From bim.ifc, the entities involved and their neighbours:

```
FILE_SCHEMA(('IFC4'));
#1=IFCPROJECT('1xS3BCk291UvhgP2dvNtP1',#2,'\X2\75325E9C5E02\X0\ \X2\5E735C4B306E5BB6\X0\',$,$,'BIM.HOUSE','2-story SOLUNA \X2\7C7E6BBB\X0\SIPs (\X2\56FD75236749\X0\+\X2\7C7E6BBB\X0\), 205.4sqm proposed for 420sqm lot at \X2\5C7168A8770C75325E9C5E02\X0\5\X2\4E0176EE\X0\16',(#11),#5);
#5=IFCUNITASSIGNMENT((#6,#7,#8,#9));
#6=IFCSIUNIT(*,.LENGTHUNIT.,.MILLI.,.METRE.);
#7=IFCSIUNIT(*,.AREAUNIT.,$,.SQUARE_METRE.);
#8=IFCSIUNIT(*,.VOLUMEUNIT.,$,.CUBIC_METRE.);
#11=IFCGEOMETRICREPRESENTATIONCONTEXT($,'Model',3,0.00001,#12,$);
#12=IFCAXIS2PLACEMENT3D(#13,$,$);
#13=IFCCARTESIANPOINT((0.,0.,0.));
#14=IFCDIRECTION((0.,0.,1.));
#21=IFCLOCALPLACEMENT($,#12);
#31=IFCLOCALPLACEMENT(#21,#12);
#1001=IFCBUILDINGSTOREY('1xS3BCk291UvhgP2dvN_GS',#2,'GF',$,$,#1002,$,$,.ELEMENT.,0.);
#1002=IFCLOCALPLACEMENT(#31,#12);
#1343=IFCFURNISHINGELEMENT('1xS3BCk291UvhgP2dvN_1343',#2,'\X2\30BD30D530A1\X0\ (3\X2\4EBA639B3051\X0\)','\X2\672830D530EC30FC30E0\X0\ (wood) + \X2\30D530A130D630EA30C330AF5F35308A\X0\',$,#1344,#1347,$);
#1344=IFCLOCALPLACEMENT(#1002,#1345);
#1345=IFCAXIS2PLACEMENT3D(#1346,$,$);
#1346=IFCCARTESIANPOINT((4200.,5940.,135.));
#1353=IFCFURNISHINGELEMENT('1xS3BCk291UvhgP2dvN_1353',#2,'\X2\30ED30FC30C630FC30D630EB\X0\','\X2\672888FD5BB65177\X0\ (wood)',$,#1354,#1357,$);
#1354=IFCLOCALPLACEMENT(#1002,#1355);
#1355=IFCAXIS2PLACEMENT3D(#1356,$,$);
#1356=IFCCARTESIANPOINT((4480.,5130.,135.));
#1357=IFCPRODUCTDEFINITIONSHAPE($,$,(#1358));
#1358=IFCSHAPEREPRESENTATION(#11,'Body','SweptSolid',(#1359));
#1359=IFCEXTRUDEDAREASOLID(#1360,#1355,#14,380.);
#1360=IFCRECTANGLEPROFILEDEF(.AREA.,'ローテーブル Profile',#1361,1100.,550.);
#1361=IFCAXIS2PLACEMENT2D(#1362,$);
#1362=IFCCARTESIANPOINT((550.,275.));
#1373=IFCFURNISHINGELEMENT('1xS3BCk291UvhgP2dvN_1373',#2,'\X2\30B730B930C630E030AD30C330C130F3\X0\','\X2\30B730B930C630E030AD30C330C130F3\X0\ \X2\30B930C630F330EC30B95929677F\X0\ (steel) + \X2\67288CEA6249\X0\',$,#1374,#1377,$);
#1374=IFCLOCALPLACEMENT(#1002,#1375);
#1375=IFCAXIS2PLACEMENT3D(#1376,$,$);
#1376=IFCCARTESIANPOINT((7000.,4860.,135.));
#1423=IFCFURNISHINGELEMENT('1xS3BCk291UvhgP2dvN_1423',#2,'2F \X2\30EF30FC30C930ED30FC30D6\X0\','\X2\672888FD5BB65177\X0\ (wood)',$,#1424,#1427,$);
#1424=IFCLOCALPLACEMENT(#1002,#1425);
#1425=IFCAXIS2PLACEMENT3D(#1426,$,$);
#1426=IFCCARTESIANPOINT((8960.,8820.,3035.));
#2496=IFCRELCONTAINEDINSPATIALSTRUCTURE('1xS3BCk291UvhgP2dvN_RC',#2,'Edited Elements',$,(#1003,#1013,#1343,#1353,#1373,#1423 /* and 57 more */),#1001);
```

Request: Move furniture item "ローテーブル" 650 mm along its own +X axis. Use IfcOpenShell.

```python
import ifcopenshell
import ifcopenshell.api.geometry
import ifcopenshell.util.placement

model = ifcopenshell.open("bim.ifc")

item = model.by_guid("1xS3BCk291UvhgP2dvN_1353")
matrix = ifcopenshell.util.placement.get_local_placement(item.ObjectPlacement)
matrix[:3, 3] += matrix[:3, 0] * 650.0
ifcopenshell.api.geometry.edit_object_placement(model, product=item, matrix=matrix, is_si=False)

print(ifcopenshell.util.placement.get_local_placement(item.ObjectPlacement).round(3) + 0.0)

model.write("bim_rev.ifc")
```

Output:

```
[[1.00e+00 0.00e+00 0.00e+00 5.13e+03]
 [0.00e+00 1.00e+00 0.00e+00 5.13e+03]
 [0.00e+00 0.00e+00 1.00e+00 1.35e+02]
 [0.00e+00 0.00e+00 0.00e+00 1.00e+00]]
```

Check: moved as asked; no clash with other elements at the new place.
